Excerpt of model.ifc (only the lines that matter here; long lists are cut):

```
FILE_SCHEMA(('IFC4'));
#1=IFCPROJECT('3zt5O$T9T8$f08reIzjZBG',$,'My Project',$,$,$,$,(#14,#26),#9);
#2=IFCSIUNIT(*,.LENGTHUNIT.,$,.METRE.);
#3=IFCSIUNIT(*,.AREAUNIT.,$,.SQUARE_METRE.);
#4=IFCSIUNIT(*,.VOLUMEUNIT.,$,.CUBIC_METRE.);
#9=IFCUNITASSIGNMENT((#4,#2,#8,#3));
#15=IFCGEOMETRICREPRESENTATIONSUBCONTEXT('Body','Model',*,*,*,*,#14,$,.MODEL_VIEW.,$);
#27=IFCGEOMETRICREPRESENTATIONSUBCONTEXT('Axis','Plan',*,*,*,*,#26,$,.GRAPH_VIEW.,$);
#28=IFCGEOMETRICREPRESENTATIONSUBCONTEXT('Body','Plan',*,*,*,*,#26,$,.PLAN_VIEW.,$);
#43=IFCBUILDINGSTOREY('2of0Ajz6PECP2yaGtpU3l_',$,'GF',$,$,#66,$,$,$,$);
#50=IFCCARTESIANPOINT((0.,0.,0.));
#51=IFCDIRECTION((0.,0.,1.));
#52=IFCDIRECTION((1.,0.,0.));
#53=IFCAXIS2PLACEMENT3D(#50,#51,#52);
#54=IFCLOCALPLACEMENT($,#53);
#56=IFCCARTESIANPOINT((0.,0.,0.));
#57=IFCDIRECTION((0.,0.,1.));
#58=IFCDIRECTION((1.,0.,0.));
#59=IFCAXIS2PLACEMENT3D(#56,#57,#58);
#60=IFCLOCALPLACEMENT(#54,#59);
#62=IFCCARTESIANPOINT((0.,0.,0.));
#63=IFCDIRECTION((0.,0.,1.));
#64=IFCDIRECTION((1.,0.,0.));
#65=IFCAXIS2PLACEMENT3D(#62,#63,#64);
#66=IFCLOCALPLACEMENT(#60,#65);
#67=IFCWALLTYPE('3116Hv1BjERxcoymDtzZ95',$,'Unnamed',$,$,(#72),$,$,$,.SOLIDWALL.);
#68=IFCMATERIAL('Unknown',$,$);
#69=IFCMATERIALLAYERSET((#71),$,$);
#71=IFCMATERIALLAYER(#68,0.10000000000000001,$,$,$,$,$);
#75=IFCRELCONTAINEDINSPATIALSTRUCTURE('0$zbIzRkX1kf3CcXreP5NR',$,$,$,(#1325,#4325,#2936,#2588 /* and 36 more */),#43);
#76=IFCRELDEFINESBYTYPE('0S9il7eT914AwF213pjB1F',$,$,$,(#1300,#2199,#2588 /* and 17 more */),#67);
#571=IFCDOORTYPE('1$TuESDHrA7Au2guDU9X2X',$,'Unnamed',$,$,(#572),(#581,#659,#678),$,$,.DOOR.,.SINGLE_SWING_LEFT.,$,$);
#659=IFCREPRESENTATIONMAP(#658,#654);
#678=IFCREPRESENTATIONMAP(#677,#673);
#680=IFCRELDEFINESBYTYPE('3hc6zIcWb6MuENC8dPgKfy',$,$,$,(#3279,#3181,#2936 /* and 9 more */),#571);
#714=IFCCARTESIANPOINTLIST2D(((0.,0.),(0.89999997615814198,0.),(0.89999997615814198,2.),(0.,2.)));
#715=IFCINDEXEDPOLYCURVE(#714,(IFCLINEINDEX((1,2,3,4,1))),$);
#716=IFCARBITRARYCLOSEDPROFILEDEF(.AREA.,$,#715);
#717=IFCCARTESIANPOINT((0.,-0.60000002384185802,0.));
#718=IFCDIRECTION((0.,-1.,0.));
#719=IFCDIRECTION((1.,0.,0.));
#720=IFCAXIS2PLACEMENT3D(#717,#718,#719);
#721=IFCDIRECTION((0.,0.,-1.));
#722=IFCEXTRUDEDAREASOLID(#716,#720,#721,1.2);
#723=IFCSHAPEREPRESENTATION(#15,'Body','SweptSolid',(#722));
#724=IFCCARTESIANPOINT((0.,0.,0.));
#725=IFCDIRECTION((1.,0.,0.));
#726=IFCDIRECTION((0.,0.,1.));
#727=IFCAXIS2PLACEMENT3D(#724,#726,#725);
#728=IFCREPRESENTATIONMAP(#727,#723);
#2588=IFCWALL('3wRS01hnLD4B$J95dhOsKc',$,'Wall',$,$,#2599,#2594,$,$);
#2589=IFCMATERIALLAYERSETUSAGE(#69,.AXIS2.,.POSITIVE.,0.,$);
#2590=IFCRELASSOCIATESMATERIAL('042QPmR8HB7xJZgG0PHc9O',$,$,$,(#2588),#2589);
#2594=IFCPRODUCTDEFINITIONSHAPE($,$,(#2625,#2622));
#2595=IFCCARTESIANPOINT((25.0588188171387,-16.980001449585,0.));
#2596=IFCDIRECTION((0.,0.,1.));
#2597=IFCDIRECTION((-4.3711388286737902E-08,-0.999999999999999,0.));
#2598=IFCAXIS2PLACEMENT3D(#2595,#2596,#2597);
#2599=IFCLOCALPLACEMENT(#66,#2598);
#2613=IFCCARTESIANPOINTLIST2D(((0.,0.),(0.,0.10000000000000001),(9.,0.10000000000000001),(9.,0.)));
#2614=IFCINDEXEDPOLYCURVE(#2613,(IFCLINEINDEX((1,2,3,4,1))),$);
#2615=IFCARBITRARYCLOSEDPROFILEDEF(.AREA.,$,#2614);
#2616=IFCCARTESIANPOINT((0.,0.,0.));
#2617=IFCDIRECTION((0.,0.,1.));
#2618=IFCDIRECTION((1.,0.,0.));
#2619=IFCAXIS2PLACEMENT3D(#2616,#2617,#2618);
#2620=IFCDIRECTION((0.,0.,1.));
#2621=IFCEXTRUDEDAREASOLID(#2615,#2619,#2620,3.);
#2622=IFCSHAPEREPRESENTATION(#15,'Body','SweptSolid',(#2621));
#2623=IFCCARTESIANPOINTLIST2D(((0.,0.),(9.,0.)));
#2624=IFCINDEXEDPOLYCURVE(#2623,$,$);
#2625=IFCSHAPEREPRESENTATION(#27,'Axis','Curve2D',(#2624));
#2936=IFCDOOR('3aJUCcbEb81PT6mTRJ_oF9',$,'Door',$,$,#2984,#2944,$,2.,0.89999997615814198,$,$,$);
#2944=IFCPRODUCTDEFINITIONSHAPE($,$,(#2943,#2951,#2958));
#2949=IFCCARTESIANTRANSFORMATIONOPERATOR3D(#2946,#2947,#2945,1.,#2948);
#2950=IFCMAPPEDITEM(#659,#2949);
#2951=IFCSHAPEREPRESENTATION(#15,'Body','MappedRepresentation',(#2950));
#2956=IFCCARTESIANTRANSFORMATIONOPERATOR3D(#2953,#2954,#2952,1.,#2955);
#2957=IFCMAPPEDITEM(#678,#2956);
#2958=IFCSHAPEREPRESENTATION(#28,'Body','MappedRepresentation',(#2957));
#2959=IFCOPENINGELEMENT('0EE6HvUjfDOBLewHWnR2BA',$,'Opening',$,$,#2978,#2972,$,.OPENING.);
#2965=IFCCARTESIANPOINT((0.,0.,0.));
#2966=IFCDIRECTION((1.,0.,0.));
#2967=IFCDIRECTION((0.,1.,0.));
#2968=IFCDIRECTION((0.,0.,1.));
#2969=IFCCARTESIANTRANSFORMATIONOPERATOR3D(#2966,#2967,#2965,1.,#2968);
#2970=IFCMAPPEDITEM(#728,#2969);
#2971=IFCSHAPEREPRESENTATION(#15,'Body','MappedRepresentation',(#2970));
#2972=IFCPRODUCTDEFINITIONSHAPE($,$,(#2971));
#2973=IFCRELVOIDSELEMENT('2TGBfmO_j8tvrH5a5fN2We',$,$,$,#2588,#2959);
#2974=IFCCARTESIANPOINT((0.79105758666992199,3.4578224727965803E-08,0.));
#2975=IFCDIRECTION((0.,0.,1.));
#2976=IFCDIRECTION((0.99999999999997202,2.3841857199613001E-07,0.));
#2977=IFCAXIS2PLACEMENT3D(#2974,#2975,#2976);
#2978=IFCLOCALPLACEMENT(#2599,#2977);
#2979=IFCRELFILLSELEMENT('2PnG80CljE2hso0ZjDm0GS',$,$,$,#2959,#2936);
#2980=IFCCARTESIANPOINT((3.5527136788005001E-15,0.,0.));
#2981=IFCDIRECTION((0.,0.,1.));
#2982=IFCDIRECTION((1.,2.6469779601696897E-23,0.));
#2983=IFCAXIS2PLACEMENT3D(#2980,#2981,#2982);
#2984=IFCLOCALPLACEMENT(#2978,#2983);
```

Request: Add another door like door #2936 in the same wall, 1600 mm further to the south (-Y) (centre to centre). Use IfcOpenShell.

```python
import ifcopenshell
import ifcopenshell.api.feature
import ifcopenshell.api.geometry
import ifcopenshell.api.root
import ifcopenshell.geom
import ifcopenshell.util.element
import ifcopenshell.util.placement
import ifcopenshell.util.shape
import ifcopenshell.util.unit

model = ifcopenshell.open("model.ifc")
unit_scale = ifcopenshell.util.unit.calculate_unit_scale(model)
settings = ifcopenshell.geom.settings()


def volume(element):
    """Net volume in cubic metres, openings subtracted."""
    shape = ifcopenshell.geom.create_shape(settings, element)
    return ifcopenshell.util.shape.get_volume(shape.geometry)


door = model.by_guid("3aJUCcbEb81PT6mTRJ_oF9")
opening = door.FillsVoids[0].RelatingOpeningElement
wall = opening.VoidsElements[0].RelatingBuildingElement
before = volume(wall)
shift = ifcopenshell.util.placement.get_local_placement(wall.ObjectPlacement)[:3, 0] * 1.6 / unit_scale

# copy_class copies the void relationship, type, container and properties, but no geometry.
new_opening = ifcopenshell.api.root.copy_class(model, product=opening)
new_opening.Representation = ifcopenshell.util.element.copy_deep(
    model, opening.Representation, exclude=["IfcGeometricRepresentationContext", "IfcRepresentationMap"]
)
new_door = ifcopenshell.api.root.copy_class(model, product=door)
new_door.Representation = ifcopenshell.util.element.copy_deep(
    model, door.Representation, exclude=["IfcGeometricRepresentationContext", "IfcRepresentationMap"]
)
ifcopenshell.api.feature.add_filling(model, opening=new_opening, element=new_door)

for old, new in ((opening, new_opening), (door, new_door)):
    matrix = ifcopenshell.util.placement.get_local_placement(old.ObjectPlacement)
    matrix[:3, 3] += shift
    ifcopenshell.api.geometry.edit_object_placement(model, product=new, matrix=matrix, is_si=False)

after = volume(wall)

print(f"wall volume {before:.3f} -> {after:.3f} m3")

model.write("model_edited.ifc")
```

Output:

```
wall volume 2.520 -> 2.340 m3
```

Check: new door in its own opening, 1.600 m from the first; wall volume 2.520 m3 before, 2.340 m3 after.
